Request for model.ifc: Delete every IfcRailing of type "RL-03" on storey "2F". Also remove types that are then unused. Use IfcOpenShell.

First a look at what the model holds.

```python
import ifcopenshell
import ifcopenshell.util.element

model = ifcopenshell.open("model.ifc")
print(model.schema)
storey = next(s for s in model.by_type("IfcBuildingStorey") if s.Name == "2F")
railings = [e for e in ifcopenshell.util.element.get_decomposition(storey) if e.is_a("IfcRailing")]
seen = {}
for e in railings:
    element_type = ifcopenshell.util.element.get_type(e)
    name = element_type.Name if element_type not in (None, e) else None
    seen[name] = seen.get(name, 0) + 1
for name, count in sorted(seen.items(), key=str):
    print(count, "x", name)
```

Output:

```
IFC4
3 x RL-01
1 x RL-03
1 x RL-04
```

```python
import ifcopenshell
import ifcopenshell.api.root
import ifcopenshell.util.element

model = ifcopenshell.open("model.ifc")

storey = next(s for s in model.by_type("IfcBuildingStorey") if s.Name == "2F")
railings = [e for e in ifcopenshell.util.element.get_decomposition(storey) if e.is_a("IfcRailing")]
targets = [e for e in railings if (t := ifcopenshell.util.element.get_type(e)) not in (None, e) and t.Name == "RL-03"]
types = {ifcopenshell.util.element.get_type(e) for e in targets} - {None, *targets}

for e in targets:
    ifcopenshell.api.root.remove_product(model, product=e)
print(len(targets), "removed")

unused = [t for t in types if not ifcopenshell.util.element.get_types(t)]
for t in unused:
    ifcopenshell.api.root.remove_product(model, product=t)
print(len(unused), "unused types removed")

model.write("model_updated.ifc")
```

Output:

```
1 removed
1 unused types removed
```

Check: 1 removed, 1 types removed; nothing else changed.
